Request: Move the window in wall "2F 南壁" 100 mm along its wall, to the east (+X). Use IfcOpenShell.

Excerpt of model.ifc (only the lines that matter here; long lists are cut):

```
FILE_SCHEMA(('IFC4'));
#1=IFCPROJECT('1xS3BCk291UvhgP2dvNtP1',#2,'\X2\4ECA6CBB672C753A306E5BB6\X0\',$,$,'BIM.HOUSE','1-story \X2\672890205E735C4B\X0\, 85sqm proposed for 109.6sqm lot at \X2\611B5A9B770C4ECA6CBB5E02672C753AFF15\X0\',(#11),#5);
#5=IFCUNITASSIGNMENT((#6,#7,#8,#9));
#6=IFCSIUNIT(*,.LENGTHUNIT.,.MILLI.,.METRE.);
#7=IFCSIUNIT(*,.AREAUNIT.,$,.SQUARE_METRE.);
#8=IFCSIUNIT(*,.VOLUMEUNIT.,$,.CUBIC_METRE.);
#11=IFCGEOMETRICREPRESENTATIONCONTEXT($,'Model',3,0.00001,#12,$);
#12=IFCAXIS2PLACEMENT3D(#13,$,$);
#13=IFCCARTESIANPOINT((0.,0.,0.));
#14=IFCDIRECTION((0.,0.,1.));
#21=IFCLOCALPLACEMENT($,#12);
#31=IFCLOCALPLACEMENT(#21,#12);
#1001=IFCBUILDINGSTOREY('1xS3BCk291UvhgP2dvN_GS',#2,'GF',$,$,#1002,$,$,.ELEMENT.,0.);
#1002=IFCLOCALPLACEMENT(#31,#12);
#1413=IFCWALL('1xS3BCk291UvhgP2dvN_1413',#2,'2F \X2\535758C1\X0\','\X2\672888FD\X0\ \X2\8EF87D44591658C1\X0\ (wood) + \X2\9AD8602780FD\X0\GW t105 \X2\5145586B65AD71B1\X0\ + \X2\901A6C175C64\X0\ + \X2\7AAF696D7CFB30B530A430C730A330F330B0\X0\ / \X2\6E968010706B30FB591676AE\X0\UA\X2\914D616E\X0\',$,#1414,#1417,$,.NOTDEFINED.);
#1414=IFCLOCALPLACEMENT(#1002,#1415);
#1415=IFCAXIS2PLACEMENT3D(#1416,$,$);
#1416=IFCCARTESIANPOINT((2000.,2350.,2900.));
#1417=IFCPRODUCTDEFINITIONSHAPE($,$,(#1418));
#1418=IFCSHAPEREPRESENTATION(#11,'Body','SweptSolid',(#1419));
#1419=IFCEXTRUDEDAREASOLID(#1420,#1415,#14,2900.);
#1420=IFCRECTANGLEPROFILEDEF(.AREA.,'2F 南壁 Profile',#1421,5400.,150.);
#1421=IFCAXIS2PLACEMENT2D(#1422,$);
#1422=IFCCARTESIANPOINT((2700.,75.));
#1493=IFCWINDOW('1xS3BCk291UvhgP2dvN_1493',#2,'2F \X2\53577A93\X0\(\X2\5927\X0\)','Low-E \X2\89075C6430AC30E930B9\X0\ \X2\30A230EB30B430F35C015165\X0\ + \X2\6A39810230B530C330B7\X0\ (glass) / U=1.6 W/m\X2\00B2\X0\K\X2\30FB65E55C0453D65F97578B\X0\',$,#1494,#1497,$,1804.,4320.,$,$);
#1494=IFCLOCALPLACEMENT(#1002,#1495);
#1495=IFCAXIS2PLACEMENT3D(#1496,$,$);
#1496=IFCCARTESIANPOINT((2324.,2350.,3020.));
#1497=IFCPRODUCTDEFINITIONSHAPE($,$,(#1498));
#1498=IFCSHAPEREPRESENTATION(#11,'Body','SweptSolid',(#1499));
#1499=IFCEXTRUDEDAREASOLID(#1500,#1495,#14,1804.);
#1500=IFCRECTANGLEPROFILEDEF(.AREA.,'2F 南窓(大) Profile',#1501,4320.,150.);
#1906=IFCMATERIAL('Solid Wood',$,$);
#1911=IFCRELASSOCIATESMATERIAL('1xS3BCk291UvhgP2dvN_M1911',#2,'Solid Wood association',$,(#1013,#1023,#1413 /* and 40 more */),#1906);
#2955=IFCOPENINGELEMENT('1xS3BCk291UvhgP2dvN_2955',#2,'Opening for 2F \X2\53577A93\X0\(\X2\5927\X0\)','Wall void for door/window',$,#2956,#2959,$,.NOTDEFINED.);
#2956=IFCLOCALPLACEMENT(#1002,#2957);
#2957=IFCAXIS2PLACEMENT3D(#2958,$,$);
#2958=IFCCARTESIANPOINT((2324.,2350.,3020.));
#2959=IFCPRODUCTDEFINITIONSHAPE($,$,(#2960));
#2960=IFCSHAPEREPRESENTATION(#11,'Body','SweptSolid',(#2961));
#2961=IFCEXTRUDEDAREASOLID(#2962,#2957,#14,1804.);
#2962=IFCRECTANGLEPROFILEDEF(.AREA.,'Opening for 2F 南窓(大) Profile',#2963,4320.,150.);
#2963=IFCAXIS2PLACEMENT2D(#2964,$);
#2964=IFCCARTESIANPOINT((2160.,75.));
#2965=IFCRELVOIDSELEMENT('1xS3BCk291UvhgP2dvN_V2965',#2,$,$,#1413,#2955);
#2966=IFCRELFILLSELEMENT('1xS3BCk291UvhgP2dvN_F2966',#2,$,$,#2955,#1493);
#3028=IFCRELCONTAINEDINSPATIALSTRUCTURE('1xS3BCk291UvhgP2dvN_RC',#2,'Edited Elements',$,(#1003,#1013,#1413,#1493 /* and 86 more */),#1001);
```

```python
import ifcopenshell
import ifcopenshell.api.geometry
import ifcopenshell.util.placement

model = ifcopenshell.open("model.ifc")

window = model.by_guid("1xS3BCk291UvhgP2dvN_1493")
opening = window.FillsVoids[0].RelatingOpeningElement
wall = opening.VoidsElements[0].RelatingBuildingElement

wall_matrix = ifcopenshell.util.placement.get_local_placement(wall.ObjectPlacement)
shift = wall_matrix[:3, 0] * 100.0
before = ifcopenshell.util.placement.get_local_placement(window.ObjectPlacement)[:3, 3].copy()

# The window is not placed relative to its opening, so move both.
for product in (opening, window):
    matrix = ifcopenshell.util.placement.get_local_placement(product.ObjectPlacement)
    matrix[:3, 3] += shift
    ifcopenshell.api.geometry.edit_object_placement(model, product=product, matrix=matrix, is_si=False)

after = ifcopenshell.util.placement.get_local_placement(window.ObjectPlacement)[:3, 3]
print("window moved by", (after - before).round(3) + 0.0)

model.write("model_updated.ifc")
```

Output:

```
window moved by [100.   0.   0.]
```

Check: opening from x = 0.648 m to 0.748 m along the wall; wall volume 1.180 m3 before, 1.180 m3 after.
